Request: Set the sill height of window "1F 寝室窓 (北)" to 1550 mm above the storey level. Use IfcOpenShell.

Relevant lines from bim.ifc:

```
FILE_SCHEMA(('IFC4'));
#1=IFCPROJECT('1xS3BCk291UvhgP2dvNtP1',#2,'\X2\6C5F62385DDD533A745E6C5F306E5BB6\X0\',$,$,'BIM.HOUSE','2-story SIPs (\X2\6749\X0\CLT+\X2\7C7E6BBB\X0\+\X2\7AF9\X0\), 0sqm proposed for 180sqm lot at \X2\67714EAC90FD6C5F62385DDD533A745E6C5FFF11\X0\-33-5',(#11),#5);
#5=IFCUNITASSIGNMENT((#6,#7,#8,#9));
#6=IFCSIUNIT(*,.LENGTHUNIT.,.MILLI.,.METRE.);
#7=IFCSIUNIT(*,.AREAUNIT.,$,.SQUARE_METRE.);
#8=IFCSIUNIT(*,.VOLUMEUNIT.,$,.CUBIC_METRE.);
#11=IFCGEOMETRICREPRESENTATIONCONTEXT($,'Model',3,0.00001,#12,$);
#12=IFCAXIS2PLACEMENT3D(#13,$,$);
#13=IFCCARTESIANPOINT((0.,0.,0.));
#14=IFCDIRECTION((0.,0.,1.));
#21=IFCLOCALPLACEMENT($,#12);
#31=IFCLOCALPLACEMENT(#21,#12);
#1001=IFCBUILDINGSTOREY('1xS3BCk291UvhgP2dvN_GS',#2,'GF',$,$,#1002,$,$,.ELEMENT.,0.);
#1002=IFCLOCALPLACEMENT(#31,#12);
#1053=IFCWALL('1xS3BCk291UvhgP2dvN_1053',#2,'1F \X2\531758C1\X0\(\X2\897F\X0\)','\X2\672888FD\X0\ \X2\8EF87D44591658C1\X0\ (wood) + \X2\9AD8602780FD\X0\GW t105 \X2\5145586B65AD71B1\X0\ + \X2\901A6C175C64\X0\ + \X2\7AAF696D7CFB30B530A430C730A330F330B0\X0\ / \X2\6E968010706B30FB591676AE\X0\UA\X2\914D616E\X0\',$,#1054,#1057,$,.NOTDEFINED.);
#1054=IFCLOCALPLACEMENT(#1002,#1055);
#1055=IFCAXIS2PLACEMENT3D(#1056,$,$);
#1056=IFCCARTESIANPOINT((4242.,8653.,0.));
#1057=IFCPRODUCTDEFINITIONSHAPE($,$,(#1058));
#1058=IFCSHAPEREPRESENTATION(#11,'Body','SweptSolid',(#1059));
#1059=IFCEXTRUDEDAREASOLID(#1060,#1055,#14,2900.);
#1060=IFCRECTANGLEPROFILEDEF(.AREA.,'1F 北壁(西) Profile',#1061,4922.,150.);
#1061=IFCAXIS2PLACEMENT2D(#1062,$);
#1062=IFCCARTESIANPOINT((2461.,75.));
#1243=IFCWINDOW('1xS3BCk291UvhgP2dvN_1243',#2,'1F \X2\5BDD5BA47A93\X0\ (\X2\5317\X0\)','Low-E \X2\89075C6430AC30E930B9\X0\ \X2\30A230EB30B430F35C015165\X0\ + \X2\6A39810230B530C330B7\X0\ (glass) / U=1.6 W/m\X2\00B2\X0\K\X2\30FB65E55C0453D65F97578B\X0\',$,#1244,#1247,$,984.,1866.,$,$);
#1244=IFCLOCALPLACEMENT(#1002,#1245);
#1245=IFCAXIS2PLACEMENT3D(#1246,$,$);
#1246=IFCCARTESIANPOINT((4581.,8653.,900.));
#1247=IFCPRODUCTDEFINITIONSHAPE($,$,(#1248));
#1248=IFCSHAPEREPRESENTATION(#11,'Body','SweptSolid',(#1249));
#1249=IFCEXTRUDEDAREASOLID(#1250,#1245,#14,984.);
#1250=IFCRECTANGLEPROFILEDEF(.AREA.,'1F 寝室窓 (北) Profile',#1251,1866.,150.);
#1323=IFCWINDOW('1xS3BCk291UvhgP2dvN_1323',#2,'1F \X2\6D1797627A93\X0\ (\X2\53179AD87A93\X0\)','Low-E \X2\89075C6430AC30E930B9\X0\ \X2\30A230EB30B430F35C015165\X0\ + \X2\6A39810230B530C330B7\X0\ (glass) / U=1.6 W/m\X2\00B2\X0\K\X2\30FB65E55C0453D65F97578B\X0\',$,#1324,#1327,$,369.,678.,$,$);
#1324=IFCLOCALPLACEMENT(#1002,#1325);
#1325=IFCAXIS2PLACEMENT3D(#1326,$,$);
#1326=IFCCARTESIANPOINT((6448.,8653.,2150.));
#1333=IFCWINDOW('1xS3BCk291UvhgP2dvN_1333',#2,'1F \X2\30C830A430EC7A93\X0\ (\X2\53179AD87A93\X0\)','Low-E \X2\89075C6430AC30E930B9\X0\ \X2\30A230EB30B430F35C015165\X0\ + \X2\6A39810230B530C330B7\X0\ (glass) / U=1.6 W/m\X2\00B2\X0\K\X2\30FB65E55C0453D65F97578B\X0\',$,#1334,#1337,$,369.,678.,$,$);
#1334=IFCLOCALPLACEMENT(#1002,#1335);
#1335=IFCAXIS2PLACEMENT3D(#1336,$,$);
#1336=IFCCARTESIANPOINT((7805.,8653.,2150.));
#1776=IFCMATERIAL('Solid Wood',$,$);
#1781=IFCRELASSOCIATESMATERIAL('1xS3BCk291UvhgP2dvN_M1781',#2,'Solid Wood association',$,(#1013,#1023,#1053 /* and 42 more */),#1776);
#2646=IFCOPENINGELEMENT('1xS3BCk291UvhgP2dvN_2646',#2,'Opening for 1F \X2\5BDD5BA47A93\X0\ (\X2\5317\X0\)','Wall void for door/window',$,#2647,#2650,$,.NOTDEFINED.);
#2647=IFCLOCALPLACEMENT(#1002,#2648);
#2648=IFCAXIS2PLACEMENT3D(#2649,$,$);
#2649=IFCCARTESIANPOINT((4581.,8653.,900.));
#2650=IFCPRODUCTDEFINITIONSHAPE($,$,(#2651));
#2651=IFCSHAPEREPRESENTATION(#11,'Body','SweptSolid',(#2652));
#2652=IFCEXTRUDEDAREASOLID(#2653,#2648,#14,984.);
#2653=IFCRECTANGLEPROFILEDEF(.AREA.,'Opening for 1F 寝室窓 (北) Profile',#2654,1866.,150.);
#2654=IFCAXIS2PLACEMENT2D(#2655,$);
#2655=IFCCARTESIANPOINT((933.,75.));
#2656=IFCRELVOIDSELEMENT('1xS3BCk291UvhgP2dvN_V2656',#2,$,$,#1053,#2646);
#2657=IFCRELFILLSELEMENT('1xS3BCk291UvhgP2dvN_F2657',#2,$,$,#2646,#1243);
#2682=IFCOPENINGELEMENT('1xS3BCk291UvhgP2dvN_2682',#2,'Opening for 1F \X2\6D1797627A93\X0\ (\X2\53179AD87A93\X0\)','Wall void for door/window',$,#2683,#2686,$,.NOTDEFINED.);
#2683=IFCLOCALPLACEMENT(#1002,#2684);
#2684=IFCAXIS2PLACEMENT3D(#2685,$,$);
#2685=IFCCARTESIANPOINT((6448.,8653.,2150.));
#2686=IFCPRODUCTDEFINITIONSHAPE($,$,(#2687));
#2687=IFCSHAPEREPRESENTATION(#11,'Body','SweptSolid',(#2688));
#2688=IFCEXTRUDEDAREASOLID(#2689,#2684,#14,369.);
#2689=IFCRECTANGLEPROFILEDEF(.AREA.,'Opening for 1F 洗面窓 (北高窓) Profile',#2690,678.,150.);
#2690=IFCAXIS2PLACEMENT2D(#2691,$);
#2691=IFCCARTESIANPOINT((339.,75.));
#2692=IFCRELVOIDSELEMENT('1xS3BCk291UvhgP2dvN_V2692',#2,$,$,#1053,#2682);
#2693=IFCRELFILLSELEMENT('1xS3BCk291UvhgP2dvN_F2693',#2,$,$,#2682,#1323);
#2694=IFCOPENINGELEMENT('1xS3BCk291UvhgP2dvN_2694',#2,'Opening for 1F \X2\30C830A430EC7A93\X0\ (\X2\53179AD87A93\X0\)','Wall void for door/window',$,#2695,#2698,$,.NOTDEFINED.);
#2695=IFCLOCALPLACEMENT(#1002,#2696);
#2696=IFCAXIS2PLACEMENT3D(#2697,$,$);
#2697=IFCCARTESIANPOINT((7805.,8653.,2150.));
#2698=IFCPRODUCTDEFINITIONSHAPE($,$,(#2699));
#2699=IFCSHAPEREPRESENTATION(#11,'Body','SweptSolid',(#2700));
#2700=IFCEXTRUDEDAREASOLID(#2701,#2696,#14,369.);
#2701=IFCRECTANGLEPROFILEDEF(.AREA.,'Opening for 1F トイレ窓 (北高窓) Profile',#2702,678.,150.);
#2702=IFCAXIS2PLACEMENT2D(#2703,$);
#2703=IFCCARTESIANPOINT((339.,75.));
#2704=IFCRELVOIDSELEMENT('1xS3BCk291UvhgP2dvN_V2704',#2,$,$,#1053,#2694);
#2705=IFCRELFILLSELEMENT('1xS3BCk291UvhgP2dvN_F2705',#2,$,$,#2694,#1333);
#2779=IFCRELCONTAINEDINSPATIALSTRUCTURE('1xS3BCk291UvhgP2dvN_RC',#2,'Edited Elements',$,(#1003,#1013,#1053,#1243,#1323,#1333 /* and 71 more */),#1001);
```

```python
import numpy as np
import ifcopenshell
import ifcopenshell.api.geometry
import ifcopenshell.geom
import ifcopenshell.util.element
import ifcopenshell.util.placement
import ifcopenshell.util.shape
import ifcopenshell.util.unit

model = ifcopenshell.open("bim.ifc")
unit_scale = ifcopenshell.util.unit.calculate_unit_scale(model)

window = model.by_guid("1xS3BCk291UvhgP2dvN_1243")
opening = window.FillsVoids[0].RelatingOpeningElement
storey = ifcopenshell.util.element.get_container(window, ifc_class="IfcBuildingStorey")
level = ifcopenshell.util.placement.get_local_placement(storey.ObjectPlacement)[2, 3]

# The opening's origin need not be at the sill, so measure its lowest point.
shape = ifcopenshell.geom.create_shape(ifcopenshell.geom.settings(), opening)
bottom = ifcopenshell.util.shape.get_shape_bottom_elevation(shape, shape.geometry) / unit_scale
dz = level + 1550.0 - bottom

shift = np.array([0.0, 0.0, dz])
# The window is not placed relative to its opening, so move both.
for product in (opening, window):
    matrix = ifcopenshell.util.placement.get_local_placement(product.ObjectPlacement)
    matrix[:3, 3] += shift
    ifcopenshell.api.geometry.edit_object_placement(model, product=product, matrix=matrix, is_si=False)

print(f"moved by {dz * unit_scale:+.3f} m")

model.write("bim_v2.ifc")
```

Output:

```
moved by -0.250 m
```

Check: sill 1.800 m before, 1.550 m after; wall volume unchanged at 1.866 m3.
